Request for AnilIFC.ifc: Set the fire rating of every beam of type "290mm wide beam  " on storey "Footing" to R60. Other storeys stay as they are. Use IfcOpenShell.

First a look at what the model holds.

```python
import ifcopenshell
import ifcopenshell.util.element

model = ifcopenshell.open("AnilIFC.ifc")
print(model.schema)
storey = next(s for s in model.by_type("IfcBuildingStorey") if s.Name == "Footing")
beams = [e for e in ifcopenshell.util.element.get_decomposition(storey) if e.is_a("IfcBeam")]
seen = {}
for e in beams:
    element_type = ifcopenshell.util.element.get_type(e)
    key = (element_type.Name if element_type != e and element_type else None, ifcopenshell.util.element.get_pset(e, "Pset_BeamCommon", "FireRating"))
    seen[key] = seen.get(key, 0) + 1
for (name, value), count in sorted(seen.items(), key=str):
    print(count, "x", name, "|", value)
```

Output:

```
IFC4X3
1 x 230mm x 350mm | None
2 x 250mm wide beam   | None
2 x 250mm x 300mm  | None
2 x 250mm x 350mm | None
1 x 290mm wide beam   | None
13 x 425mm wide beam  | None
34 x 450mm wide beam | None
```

```python
import ifcopenshell
import ifcopenshell.api.pset
import ifcopenshell.util.element

model = ifcopenshell.open("AnilIFC.ifc")

storey = next(s for s in model.by_type("IfcBuildingStorey") if s.Name == "Footing")
beams = [e for e in ifcopenshell.util.element.get_decomposition(storey) if e.is_a("IfcBeam")]

count = 0
for e in beams:
    element_type = ifcopenshell.util.element.get_type(e)
    if element_type in (None, e) or element_type.Name != "290mm wide beam  ":
        continue
    # add_pset returns the element's existing set when there is one.
    pset = ifcopenshell.api.pset.add_pset(model, product=e, name="Pset_BeamCommon")
    ifcopenshell.api.pset.edit_pset(model, pset=pset, properties={"FireRating": "R60"})
    count += 1

print(count, "beams updated")

model.write("AnilIFC_edited.ifc")
```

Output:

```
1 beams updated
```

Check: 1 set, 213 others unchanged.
